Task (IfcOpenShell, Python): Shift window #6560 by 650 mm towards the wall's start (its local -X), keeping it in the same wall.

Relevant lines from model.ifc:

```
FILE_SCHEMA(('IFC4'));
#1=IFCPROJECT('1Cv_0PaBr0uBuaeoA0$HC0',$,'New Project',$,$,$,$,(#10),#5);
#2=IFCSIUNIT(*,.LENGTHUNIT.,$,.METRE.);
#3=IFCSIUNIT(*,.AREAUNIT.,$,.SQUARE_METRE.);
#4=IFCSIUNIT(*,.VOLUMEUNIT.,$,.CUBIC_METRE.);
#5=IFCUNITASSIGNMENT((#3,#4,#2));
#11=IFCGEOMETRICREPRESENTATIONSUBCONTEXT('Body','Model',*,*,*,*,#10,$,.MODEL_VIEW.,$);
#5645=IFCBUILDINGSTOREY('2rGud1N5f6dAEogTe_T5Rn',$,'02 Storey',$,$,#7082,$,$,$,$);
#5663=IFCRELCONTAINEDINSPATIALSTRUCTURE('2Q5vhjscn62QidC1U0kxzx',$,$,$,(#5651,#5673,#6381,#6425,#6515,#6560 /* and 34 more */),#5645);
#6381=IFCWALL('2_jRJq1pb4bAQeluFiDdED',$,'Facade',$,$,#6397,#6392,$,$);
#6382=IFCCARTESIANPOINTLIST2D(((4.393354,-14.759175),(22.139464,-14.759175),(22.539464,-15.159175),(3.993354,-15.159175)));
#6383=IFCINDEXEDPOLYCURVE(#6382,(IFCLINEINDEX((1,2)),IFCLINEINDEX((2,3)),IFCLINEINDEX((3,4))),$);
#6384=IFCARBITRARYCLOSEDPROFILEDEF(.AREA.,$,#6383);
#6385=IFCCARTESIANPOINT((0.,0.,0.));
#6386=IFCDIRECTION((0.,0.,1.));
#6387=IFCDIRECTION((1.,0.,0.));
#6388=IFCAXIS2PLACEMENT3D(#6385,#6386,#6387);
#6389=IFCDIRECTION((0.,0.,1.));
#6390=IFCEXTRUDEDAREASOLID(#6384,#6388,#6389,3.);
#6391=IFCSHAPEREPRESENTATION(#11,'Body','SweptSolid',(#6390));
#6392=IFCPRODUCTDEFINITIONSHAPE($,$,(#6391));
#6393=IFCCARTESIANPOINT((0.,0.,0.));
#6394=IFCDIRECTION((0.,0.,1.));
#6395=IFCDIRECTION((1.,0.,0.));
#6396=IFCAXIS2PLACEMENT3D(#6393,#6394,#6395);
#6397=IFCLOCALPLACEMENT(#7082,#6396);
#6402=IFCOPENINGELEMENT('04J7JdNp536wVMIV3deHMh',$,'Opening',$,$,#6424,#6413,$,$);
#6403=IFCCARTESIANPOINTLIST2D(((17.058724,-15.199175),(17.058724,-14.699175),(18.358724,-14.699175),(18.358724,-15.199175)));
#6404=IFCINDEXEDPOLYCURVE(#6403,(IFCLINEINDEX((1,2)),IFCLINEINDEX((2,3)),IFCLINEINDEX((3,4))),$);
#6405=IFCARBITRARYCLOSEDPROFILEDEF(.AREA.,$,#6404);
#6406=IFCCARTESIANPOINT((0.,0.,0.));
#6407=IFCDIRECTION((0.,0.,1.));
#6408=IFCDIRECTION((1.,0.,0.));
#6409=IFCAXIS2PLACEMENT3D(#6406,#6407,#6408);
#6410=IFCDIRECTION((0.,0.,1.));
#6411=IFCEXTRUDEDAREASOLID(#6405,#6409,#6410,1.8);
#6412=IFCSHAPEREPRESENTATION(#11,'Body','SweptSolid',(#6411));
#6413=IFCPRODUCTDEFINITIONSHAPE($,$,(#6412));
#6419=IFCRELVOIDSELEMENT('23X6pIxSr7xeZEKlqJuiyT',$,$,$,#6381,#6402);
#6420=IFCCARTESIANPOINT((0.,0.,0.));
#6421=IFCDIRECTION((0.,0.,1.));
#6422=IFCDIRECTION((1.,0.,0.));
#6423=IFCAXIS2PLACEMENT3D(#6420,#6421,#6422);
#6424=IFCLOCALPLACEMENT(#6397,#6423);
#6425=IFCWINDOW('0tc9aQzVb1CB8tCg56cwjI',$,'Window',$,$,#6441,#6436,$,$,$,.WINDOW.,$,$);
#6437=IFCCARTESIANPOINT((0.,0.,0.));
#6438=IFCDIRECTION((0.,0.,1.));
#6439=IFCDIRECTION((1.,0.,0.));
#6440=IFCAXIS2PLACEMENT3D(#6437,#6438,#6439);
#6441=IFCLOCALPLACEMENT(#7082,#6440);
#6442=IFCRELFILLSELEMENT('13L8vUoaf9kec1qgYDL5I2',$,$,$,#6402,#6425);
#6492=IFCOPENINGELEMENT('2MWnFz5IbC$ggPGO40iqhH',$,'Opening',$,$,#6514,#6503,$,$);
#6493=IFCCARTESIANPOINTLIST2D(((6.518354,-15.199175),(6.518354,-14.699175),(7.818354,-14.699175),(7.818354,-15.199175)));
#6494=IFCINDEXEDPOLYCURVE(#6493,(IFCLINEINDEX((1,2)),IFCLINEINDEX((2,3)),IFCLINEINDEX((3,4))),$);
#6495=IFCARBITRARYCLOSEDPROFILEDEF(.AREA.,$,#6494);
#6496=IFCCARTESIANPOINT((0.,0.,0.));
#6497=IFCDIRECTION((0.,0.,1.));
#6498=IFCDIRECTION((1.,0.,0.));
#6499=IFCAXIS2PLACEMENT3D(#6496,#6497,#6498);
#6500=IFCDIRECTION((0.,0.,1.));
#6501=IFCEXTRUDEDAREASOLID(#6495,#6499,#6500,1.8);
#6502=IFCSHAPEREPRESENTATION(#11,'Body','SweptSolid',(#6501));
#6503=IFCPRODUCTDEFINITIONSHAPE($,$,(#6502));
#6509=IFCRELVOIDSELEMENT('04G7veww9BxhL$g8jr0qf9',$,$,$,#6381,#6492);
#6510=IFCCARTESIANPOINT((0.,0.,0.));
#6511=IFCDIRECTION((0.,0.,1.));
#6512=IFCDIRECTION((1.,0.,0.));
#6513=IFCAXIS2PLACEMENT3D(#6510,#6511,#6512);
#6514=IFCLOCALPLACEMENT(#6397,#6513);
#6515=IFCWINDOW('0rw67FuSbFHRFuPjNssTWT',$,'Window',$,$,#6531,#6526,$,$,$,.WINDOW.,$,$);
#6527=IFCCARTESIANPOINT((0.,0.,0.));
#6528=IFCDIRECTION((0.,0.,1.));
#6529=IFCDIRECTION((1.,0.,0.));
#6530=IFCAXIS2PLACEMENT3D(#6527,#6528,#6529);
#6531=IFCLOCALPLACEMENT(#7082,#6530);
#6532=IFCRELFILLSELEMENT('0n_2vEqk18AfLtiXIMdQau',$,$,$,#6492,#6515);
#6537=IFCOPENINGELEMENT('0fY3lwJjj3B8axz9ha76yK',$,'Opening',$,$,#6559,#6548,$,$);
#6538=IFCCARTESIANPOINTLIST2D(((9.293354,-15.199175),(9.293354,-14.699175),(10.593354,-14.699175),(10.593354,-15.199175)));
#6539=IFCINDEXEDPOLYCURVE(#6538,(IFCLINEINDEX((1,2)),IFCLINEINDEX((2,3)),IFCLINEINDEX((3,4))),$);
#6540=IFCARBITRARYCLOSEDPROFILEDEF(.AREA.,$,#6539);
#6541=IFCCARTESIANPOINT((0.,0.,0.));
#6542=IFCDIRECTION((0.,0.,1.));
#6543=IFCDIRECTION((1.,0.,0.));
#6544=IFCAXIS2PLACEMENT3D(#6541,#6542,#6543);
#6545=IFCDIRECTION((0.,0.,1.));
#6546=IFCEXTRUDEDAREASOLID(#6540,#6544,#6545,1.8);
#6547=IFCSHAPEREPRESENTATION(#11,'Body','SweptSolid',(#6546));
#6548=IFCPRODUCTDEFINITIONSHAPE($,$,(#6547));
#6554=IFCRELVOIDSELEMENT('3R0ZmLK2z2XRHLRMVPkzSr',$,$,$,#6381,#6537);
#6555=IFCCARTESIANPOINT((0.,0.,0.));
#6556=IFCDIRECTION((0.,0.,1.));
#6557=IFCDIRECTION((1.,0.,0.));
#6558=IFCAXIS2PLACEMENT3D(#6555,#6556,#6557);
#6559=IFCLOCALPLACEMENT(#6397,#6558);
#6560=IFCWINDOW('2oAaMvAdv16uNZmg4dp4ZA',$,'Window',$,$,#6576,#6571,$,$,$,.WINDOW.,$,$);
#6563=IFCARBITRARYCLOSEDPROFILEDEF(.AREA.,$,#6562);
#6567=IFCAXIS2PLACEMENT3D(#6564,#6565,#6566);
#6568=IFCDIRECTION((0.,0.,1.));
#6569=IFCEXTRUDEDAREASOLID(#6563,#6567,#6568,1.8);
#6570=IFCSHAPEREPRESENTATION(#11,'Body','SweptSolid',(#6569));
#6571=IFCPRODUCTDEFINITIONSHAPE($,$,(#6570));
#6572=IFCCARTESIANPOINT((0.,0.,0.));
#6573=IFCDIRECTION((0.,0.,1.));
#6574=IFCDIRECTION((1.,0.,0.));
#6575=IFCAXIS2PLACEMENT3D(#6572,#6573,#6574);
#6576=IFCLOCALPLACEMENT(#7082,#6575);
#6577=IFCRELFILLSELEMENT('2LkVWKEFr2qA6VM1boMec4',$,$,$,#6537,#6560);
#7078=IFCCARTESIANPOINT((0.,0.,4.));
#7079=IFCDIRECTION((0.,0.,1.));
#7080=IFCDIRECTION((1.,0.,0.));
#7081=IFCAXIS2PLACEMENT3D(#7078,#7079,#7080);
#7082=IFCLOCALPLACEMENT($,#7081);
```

```python
import ifcopenshell
import ifcopenshell.api.geometry
import ifcopenshell.util.placement
import ifcopenshell.util.unit

model = ifcopenshell.open("model.ifc")
unit_scale = ifcopenshell.util.unit.calculate_unit_scale(model)

window = model.by_guid("2oAaMvAdv16uNZmg4dp4ZA")
opening = window.FillsVoids[0].RelatingOpeningElement
wall = opening.VoidsElements[0].RelatingBuildingElement

wall_matrix = ifcopenshell.util.placement.get_local_placement(wall.ObjectPlacement)
shift = wall_matrix[:3, 0] * -0.65 / unit_scale
before = ifcopenshell.util.placement.get_local_placement(window.ObjectPlacement)[:3, 3].copy()

# The window is not placed relative to its opening, so move both.
for product in (opening, window):
    matrix = ifcopenshell.util.placement.get_local_placement(product.ObjectPlacement)
    matrix[:3, 3] += shift
    ifcopenshell.api.geometry.edit_object_placement(model, product=product, matrix=matrix, is_si=False)

after = ifcopenshell.util.placement.get_local_placement(window.ObjectPlacement)[:3, 3]
print("window moved by", (after - before).round(3) + 0.0)

model.write("model-out.ifc")
```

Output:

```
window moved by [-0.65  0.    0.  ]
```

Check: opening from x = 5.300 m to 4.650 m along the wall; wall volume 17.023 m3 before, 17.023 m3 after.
